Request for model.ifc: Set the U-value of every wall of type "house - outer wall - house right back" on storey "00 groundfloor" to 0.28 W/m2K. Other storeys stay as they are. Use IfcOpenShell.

First a look at what the model holds.

```python
import ifcopenshell
import ifcopenshell.util.element

model = ifcopenshell.open("model.ifc")
print(model.schema)
storey = next(s for s in model.by_type("IfcBuildingStorey") if s.Name == "00 groundfloor")
walls = [e for e in ifcopenshell.util.element.get_decomposition(storey) if e.is_a("IfcWall")]
seen = {}
for e in walls:
    element_type = ifcopenshell.util.element.get_type(e)
    key = (element_type.Name if element_type != e and element_type else None, ifcopenshell.util.element.get_pset(e, "Pset_WallCommon", "ThermalTransmittance"))
    seen[key] = seen.get(key, 0) + 1
for (name, value), count in sorted(seen.items(), key=str):
    print(count, "x", name, "|", value)
```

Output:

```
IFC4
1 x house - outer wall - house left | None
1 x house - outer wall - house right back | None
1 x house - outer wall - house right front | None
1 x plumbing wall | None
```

```python
import ifcopenshell
import ifcopenshell.api.pset
import ifcopenshell.util.element

model = ifcopenshell.open("model.ifc")

storey = next(s for s in model.by_type("IfcBuildingStorey") if s.Name == "00 groundfloor")
walls = [e for e in ifcopenshell.util.element.get_decomposition(storey) if e.is_a("IfcWall")]

count = 0
for e in walls:
    element_type = ifcopenshell.util.element.get_type(e)
    if element_type in (None, e) or element_type.Name != "house - outer wall - house right back":
        continue
    # add_pset returns the element's existing set when there is one.
    pset = ifcopenshell.api.pset.add_pset(model, product=e, name="Pset_WallCommon")
    ifcopenshell.api.pset.edit_pset(model, pset=pset, properties={"ThermalTransmittance": 0.28})
    count += 1

print(count, "walls updated")

model.write("model_rev.ifc")
```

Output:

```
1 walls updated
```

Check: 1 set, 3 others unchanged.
